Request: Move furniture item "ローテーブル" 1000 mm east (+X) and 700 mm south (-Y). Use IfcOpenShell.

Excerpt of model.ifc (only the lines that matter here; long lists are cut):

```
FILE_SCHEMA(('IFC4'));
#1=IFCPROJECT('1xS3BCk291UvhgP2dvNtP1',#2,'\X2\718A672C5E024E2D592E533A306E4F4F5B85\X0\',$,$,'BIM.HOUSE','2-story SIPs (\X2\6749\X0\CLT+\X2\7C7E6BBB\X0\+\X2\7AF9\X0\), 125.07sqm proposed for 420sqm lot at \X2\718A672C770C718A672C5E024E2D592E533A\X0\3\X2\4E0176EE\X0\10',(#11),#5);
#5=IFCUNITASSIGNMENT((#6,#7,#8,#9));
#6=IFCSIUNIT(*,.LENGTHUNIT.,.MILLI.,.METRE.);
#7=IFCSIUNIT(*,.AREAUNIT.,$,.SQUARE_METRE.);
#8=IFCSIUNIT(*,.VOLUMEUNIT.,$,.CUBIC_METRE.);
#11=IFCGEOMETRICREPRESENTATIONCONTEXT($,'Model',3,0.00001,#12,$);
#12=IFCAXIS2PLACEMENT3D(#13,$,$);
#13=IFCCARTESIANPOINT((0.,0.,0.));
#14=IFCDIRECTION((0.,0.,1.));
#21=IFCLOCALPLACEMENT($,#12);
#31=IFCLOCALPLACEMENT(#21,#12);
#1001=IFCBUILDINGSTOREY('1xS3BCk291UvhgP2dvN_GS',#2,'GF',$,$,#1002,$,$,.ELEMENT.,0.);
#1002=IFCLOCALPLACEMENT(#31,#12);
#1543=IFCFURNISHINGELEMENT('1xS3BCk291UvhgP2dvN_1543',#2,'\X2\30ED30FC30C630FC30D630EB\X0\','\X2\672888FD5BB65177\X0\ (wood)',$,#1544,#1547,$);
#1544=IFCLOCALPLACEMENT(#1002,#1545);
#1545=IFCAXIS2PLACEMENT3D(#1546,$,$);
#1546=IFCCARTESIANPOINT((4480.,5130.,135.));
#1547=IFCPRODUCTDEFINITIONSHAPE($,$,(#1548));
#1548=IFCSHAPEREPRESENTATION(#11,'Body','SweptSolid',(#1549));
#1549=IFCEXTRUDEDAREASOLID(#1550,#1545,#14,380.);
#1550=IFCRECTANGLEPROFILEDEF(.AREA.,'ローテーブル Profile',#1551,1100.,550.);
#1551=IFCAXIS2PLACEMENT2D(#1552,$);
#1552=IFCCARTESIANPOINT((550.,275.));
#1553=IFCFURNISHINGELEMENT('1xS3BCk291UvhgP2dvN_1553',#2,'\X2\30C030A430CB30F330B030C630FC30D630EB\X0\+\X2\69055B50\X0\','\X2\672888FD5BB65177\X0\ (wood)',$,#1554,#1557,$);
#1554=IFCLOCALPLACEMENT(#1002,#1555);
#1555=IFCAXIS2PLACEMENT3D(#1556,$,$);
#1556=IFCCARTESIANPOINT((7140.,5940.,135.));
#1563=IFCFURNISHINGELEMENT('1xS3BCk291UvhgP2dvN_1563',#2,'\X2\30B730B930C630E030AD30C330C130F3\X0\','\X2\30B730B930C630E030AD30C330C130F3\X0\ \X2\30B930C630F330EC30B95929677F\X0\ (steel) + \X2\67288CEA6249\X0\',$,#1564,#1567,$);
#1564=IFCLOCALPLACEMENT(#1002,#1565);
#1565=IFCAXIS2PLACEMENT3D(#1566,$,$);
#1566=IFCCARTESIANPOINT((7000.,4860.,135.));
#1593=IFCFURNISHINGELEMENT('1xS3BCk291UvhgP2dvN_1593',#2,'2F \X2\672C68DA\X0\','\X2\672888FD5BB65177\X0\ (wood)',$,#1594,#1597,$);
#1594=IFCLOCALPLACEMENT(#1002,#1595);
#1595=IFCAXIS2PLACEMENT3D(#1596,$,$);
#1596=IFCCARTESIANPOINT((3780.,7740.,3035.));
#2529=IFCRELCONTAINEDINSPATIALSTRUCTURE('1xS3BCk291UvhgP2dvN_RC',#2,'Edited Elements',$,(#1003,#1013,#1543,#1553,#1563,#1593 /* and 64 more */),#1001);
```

```python
import ifcopenshell
import ifcopenshell.api.geometry
import ifcopenshell.util.placement
import ifcopenshell.util.unit

model = ifcopenshell.open("model.ifc")
unit_scale = ifcopenshell.util.unit.calculate_unit_scale(model)

item = model.by_guid("1xS3BCk291UvhgP2dvN_1543")
matrix = ifcopenshell.util.placement.get_local_placement(item.ObjectPlacement)
matrix[0, 3] += 1 / unit_scale
matrix[1, 3] -= 0.7 / unit_scale
ifcopenshell.api.geometry.edit_object_placement(model, product=item, matrix=matrix, is_si=False)

print(ifcopenshell.util.placement.get_local_placement(item.ObjectPlacement).round(3) + 0.0)

model.write("model_rev.ifc")
```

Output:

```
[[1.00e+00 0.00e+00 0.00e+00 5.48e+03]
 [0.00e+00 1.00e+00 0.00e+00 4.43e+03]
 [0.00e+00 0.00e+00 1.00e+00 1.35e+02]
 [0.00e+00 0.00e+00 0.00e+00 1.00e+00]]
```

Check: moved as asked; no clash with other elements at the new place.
